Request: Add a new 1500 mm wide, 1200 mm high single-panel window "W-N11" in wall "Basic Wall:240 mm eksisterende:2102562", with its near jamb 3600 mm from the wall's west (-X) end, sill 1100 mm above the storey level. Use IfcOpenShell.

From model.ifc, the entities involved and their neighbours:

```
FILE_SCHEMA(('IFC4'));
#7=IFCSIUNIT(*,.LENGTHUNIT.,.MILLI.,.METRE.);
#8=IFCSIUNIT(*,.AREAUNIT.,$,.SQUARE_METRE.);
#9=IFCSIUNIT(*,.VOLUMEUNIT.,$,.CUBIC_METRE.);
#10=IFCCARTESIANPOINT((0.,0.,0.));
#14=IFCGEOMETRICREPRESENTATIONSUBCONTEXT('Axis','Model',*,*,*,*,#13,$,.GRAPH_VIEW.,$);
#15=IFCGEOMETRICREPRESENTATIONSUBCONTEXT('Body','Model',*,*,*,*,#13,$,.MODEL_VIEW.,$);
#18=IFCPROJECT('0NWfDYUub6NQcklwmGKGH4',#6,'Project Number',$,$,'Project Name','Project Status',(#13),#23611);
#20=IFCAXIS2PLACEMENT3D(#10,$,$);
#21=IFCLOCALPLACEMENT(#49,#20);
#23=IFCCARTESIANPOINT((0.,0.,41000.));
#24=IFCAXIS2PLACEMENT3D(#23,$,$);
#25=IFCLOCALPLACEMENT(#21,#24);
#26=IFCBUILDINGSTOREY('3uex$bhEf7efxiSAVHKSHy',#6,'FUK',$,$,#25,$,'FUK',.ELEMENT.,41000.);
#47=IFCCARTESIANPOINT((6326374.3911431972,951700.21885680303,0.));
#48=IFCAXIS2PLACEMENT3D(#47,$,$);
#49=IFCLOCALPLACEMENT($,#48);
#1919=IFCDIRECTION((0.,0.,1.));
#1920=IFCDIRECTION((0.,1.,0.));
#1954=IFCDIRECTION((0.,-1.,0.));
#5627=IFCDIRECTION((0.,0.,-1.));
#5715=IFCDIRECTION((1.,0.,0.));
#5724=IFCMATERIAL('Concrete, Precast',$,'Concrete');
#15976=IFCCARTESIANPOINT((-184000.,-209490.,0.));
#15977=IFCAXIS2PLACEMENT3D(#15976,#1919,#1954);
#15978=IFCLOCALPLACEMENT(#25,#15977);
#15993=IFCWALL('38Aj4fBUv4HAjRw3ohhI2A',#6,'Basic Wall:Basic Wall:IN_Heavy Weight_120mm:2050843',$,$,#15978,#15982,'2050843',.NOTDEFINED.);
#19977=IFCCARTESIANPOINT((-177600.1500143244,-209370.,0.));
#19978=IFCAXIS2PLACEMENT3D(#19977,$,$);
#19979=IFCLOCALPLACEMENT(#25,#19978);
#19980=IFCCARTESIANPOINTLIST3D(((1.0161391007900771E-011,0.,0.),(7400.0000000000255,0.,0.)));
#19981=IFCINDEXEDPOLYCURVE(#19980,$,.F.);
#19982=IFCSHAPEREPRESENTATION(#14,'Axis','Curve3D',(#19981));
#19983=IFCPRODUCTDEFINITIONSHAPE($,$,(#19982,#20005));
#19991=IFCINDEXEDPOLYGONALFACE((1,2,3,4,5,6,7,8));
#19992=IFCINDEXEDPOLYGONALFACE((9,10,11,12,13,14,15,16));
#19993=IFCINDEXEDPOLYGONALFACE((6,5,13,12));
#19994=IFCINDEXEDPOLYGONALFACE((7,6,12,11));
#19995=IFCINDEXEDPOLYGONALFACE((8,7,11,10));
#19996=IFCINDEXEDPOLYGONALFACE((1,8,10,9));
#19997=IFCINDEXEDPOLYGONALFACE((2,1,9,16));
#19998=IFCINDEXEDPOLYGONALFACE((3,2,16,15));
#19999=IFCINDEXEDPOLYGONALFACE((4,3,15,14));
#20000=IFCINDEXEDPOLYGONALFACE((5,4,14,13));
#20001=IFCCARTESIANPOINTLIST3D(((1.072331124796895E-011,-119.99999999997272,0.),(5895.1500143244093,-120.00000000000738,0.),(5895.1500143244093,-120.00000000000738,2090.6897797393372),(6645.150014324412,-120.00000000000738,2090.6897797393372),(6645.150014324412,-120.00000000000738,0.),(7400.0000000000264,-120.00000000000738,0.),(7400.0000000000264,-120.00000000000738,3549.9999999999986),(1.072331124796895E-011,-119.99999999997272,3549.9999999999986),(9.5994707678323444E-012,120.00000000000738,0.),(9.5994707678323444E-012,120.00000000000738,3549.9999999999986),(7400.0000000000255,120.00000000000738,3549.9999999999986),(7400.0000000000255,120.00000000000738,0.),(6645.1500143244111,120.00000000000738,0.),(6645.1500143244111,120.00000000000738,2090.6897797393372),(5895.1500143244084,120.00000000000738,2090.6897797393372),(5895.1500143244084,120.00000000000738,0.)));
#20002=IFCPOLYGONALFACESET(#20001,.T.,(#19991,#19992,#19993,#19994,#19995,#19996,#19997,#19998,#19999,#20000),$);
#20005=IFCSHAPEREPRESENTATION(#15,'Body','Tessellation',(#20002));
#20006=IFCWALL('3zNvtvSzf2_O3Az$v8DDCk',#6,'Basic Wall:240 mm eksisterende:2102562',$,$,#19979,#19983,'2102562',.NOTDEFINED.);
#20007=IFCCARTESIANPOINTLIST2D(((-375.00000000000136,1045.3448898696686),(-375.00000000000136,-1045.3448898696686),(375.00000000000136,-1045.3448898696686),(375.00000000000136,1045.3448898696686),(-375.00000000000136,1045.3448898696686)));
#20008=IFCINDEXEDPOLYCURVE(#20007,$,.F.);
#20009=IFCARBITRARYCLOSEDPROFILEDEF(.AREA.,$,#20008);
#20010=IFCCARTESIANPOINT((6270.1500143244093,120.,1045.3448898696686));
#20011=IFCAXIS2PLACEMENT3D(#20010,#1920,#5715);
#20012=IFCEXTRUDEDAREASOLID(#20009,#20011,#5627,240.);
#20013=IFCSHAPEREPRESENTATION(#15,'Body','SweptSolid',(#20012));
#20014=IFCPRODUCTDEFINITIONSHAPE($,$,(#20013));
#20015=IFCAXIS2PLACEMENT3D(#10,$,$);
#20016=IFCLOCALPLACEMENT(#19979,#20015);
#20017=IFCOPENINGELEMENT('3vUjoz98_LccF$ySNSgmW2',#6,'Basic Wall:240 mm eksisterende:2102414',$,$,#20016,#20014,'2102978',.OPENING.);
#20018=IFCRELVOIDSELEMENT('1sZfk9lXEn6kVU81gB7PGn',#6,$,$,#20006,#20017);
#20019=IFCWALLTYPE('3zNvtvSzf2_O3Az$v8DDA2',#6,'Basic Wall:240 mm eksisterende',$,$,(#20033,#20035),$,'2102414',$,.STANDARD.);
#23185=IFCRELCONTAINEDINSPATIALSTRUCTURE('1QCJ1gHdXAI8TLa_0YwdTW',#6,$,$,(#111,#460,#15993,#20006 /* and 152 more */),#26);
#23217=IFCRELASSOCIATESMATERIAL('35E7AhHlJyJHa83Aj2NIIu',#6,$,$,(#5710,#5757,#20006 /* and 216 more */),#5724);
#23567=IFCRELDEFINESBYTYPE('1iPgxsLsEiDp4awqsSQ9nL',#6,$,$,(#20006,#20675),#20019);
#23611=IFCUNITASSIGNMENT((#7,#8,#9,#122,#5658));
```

```python
import numpy as np
import ifcopenshell
import ifcopenshell.api.feature
import ifcopenshell.api.geometry
import ifcopenshell.api.root
import ifcopenshell.api.spatial
import ifcopenshell.geom
import ifcopenshell.util.element
import ifcopenshell.util.placement
import ifcopenshell.util.representation
import ifcopenshell.util.shape
import ifcopenshell.util.unit

model = ifcopenshell.open("model.ifc")
unit_scale = ifcopenshell.util.unit.calculate_unit_scale(model)
settings = ifcopenshell.geom.settings()


def volume(element):
    """Net volume in cubic metres, openings subtracted."""
    shape = ifcopenshell.geom.create_shape(settings, element)
    return ifcopenshell.util.shape.get_volume(shape.geometry)


wall = model.by_guid("3zNvtvSzf2_O3Az$v8DDCk")
storey = ifcopenshell.util.element.get_container(wall, ifc_class="IfcBuildingStorey")
context = ifcopenshell.util.representation.get_context(model, "Model", "Body", "MODEL_VIEW")
before = volume(wall)

width, height, from_end, sill = 1.5, 1.2, 3.6, 1.1  # metres

# The wall runs along its own X axis, and the end named is its -X end.
wall_shape = ifcopenshell.geom.create_shape(settings, wall)
x, y, z = ifcopenshell.util.shape.get_vertices(wall_shape.geometry).T
start = x.min() + from_end
face, thickness = float(y.min()), float(y.max() - y.min())
wall_matrix = ifcopenshell.util.placement.get_local_placement(wall.ObjectPlacement)
level = ifcopenshell.util.placement.get_local_placement(storey.ObjectPlacement)[2, 3]


def in_wall(x, y):
    """Placement at x, y metres in the wall's axes, at sill height."""
    matrix = wall_matrix.copy()
    matrix[:, 3] = wall_matrix @ np.array([x / unit_scale, y / unit_scale, 0.0, 1.0])
    matrix[2, 3] = level + sill / unit_scale
    return matrix


# Opening: a box that overshoots both wall faces by 50 mm.
opening = ifcopenshell.api.root.create_entity(model, ifc_class="IfcOpeningElement", predefined_type="OPENING")
box = ifcopenshell.api.geometry.add_wall_representation(
    model, context=context, length=width, height=height, thickness=thickness + 0.1
)
ifcopenshell.api.geometry.assign_representation(model, product=opening, representation=box)
ifcopenshell.api.geometry.edit_object_placement(model, product=opening, matrix=in_wall(start, face - 0.05), is_si=False)
ifcopenshell.api.feature.add_feature(model, feature=opening, element=wall)

window = ifcopenshell.api.root.create_entity(model, ifc_class="IfcWindow", name="W-N11", predefined_type="WINDOW")
window.OverallWidth, window.OverallHeight = width / unit_scale, height / unit_scale
window.PartitioningType = "SINGLE_PANEL"
body = ifcopenshell.api.geometry.add_window_representation(
    model,
    context=context,
    overall_width=window.OverallWidth,
    overall_height=window.OverallHeight,
    partition_type="SINGLE_PANEL",
)
ifcopenshell.api.geometry.assign_representation(model, product=window, representation=body)
ifcopenshell.api.spatial.assign_container(model, products=[window], relating_structure=storey)
ifcopenshell.api.feature.add_filling(model, opening=opening, element=window)

# Centre the window in the wall's thickness.
ifcopenshell.api.geometry.edit_object_placement(model, product=window, matrix=in_wall(start, face), is_si=False)
window_shape = ifcopenshell.geom.create_shape(settings, window)
depth = ifcopenshell.util.shape.get_vertices(window_shape.geometry)[:, 1]
offset = face + thickness / 2 - (depth.min() + depth.max()) / 2
ifcopenshell.api.geometry.edit_object_placement(model, product=window, matrix=in_wall(start, offset), is_si=False)

after = volume(wall)

print(f"wall volume {before:.3f} -> {after:.3f} m3")

model.write("model_updated.ifc")
```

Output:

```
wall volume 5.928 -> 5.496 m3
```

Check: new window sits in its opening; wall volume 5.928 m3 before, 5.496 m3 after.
